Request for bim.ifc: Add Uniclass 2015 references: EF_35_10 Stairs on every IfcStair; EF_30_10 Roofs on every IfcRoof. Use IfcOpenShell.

First a look at what the model holds.

```python
import ifcopenshell

model = ifcopenshell.open("bim.ifc")
print(model.schema)
print("classifications:", [c.Name for c in model.by_type("IfcClassification")])
for ifc_class in ("IfcDoor", "IfcRoof", "IfcStair", "IfcWall", "IfcWindow"):
    print(ifc_class, len(model.by_type(ifc_class)))
```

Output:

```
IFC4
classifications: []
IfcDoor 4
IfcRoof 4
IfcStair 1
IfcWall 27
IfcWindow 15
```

```python
import ifcopenshell
import ifcopenshell.api.classification

model = ifcopenshell.open("bim.ifc")

system = ifcopenshell.api.classification.add_classification(model, classification="Uniclass 2015")

codes = {
    "IfcStair": ("EF_35_10", "Stairs"),
    "IfcRoof": ("EF_30_10", "Roofs"),
}
for ifc_class, (code, name) in codes.items():
    products = model.by_type(ifc_class)
    ifcopenshell.api.classification.add_reference(
        model, products=products, classification=system, identification=code, name=name
    )
    print(code, len(products))

model.write("bim_rev.ifc")
```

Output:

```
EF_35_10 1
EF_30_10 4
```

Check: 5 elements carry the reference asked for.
